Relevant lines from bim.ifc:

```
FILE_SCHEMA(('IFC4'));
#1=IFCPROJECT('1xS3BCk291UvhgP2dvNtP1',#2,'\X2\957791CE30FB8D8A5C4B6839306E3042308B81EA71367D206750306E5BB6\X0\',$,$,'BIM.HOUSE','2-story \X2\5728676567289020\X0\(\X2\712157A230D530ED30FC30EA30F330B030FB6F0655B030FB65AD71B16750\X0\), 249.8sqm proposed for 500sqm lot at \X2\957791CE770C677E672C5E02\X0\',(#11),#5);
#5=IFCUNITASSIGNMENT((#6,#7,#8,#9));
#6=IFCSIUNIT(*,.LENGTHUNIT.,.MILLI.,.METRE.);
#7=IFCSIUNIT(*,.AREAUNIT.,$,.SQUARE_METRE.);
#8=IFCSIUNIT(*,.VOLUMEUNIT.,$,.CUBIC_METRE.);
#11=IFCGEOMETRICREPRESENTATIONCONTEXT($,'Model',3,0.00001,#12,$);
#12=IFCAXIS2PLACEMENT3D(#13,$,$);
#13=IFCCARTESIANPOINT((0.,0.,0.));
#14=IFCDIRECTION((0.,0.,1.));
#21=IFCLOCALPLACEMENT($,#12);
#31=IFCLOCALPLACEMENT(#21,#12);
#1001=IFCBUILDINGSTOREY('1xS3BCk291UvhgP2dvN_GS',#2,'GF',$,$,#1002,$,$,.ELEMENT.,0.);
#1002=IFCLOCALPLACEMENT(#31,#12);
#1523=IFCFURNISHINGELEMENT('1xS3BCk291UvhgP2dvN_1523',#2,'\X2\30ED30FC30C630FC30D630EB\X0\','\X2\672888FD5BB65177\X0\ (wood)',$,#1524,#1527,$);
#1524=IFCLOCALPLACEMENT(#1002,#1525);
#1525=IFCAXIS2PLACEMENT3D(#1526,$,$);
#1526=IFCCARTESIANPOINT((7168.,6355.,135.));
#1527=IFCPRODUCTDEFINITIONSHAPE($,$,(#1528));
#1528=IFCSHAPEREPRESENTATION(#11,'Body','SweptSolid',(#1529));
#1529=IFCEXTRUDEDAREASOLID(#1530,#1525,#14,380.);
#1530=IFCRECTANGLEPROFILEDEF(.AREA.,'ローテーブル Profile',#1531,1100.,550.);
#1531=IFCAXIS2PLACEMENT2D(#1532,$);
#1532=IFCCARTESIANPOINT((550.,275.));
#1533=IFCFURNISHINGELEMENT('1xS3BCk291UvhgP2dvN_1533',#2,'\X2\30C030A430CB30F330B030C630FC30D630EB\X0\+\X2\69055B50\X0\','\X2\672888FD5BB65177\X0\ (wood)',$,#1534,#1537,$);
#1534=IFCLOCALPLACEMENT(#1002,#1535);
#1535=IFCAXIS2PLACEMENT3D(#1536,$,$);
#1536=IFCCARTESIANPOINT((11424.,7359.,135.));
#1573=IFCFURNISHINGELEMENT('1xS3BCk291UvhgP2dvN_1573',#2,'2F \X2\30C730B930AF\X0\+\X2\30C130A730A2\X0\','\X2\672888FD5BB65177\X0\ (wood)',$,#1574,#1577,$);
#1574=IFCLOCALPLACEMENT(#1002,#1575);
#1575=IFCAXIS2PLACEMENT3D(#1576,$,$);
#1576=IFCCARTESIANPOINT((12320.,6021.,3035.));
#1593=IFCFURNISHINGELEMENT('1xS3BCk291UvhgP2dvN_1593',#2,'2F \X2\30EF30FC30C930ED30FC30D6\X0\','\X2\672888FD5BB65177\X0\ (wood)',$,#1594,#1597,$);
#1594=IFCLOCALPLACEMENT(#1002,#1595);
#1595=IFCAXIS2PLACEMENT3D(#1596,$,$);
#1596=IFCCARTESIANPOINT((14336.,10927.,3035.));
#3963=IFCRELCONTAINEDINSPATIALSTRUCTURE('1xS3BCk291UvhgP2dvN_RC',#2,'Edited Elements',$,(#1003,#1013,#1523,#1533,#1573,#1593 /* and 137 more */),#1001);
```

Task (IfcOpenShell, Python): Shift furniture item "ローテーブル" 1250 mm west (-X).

```python
import ifcopenshell
import ifcopenshell.api.geometry
import ifcopenshell.util.placement

model = ifcopenshell.open("bim.ifc")

item = model.by_guid("1xS3BCk291UvhgP2dvN_1523")
matrix = ifcopenshell.util.placement.get_local_placement(item.ObjectPlacement)
matrix[0, 3] -= 1250.0
ifcopenshell.api.geometry.edit_object_placement(model, product=item, matrix=matrix, is_si=False)

print(ifcopenshell.util.placement.get_local_placement(item.ObjectPlacement).round(3) + 0.0)

model.write("bim_updated.ifc")
```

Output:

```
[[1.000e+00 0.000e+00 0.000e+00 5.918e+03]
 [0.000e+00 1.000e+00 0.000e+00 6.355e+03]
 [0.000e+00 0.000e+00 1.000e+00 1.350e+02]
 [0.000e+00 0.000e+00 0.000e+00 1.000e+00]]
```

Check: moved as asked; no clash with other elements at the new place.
